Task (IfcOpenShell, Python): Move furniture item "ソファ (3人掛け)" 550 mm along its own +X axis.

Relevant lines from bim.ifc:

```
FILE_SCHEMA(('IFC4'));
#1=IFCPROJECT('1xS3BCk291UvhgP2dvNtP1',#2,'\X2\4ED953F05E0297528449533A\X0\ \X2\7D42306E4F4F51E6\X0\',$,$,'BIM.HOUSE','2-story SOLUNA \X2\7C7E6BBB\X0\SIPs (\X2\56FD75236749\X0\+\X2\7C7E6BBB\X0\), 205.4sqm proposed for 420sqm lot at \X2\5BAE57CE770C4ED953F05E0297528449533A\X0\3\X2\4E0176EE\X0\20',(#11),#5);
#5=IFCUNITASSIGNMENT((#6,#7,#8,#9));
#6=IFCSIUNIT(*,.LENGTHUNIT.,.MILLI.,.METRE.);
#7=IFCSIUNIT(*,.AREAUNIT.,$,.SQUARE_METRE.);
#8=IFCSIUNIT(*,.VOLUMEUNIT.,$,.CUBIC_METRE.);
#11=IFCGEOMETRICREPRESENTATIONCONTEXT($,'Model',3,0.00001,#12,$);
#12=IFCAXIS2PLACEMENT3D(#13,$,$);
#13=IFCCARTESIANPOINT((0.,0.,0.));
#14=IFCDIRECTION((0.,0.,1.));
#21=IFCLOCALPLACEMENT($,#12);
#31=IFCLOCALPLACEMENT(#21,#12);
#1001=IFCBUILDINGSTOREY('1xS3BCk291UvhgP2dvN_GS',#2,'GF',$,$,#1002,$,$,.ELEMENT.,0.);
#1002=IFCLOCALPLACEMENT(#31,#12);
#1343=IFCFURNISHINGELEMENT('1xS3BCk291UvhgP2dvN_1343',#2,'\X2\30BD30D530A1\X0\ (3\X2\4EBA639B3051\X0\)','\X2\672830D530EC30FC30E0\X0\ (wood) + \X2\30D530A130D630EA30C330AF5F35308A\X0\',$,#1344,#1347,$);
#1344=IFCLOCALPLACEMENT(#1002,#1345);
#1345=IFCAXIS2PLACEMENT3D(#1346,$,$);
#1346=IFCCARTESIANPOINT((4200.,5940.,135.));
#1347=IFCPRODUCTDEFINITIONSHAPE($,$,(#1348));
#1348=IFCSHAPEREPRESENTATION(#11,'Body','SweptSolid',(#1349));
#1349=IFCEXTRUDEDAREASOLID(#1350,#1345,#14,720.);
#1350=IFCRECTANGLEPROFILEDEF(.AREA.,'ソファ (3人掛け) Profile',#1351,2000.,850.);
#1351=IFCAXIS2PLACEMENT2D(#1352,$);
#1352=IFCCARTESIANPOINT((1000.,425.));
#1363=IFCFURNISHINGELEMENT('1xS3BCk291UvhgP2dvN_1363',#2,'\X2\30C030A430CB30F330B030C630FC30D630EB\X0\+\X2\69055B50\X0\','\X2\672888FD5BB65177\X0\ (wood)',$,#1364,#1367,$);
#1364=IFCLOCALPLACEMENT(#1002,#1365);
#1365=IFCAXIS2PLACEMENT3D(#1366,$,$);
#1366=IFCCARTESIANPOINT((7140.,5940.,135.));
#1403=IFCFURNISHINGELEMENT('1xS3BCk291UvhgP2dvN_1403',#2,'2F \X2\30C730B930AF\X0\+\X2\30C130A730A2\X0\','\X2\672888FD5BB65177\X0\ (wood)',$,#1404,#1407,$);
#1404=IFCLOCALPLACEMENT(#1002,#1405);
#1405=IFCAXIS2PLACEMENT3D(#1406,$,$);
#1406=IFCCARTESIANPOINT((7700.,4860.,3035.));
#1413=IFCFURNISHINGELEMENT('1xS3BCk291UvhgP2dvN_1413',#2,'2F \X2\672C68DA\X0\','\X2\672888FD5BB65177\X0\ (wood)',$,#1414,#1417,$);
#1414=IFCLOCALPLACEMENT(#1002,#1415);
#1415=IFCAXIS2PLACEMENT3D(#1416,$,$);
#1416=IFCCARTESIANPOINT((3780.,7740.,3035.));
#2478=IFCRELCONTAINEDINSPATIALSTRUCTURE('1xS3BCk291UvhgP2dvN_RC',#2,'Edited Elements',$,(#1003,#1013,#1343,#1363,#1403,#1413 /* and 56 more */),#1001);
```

```python
import ifcopenshell
import ifcopenshell.api.geometry
import ifcopenshell.util.placement

model = ifcopenshell.open("bim.ifc")

item = model.by_id(1343)
matrix = ifcopenshell.util.placement.get_local_placement(item.ObjectPlacement)
matrix[:3, 3] += matrix[:3, 0] * 550.0
ifcopenshell.api.geometry.edit_object_placement(model, product=item, matrix=matrix, is_si=False)

print(ifcopenshell.util.placement.get_local_placement(item.ObjectPlacement).round(3) + 0.0)

model.write("bim_rev.ifc")
```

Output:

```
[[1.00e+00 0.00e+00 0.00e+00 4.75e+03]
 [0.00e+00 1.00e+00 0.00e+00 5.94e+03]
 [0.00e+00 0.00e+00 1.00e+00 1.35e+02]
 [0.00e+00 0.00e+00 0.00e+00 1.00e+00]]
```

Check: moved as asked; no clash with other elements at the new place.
